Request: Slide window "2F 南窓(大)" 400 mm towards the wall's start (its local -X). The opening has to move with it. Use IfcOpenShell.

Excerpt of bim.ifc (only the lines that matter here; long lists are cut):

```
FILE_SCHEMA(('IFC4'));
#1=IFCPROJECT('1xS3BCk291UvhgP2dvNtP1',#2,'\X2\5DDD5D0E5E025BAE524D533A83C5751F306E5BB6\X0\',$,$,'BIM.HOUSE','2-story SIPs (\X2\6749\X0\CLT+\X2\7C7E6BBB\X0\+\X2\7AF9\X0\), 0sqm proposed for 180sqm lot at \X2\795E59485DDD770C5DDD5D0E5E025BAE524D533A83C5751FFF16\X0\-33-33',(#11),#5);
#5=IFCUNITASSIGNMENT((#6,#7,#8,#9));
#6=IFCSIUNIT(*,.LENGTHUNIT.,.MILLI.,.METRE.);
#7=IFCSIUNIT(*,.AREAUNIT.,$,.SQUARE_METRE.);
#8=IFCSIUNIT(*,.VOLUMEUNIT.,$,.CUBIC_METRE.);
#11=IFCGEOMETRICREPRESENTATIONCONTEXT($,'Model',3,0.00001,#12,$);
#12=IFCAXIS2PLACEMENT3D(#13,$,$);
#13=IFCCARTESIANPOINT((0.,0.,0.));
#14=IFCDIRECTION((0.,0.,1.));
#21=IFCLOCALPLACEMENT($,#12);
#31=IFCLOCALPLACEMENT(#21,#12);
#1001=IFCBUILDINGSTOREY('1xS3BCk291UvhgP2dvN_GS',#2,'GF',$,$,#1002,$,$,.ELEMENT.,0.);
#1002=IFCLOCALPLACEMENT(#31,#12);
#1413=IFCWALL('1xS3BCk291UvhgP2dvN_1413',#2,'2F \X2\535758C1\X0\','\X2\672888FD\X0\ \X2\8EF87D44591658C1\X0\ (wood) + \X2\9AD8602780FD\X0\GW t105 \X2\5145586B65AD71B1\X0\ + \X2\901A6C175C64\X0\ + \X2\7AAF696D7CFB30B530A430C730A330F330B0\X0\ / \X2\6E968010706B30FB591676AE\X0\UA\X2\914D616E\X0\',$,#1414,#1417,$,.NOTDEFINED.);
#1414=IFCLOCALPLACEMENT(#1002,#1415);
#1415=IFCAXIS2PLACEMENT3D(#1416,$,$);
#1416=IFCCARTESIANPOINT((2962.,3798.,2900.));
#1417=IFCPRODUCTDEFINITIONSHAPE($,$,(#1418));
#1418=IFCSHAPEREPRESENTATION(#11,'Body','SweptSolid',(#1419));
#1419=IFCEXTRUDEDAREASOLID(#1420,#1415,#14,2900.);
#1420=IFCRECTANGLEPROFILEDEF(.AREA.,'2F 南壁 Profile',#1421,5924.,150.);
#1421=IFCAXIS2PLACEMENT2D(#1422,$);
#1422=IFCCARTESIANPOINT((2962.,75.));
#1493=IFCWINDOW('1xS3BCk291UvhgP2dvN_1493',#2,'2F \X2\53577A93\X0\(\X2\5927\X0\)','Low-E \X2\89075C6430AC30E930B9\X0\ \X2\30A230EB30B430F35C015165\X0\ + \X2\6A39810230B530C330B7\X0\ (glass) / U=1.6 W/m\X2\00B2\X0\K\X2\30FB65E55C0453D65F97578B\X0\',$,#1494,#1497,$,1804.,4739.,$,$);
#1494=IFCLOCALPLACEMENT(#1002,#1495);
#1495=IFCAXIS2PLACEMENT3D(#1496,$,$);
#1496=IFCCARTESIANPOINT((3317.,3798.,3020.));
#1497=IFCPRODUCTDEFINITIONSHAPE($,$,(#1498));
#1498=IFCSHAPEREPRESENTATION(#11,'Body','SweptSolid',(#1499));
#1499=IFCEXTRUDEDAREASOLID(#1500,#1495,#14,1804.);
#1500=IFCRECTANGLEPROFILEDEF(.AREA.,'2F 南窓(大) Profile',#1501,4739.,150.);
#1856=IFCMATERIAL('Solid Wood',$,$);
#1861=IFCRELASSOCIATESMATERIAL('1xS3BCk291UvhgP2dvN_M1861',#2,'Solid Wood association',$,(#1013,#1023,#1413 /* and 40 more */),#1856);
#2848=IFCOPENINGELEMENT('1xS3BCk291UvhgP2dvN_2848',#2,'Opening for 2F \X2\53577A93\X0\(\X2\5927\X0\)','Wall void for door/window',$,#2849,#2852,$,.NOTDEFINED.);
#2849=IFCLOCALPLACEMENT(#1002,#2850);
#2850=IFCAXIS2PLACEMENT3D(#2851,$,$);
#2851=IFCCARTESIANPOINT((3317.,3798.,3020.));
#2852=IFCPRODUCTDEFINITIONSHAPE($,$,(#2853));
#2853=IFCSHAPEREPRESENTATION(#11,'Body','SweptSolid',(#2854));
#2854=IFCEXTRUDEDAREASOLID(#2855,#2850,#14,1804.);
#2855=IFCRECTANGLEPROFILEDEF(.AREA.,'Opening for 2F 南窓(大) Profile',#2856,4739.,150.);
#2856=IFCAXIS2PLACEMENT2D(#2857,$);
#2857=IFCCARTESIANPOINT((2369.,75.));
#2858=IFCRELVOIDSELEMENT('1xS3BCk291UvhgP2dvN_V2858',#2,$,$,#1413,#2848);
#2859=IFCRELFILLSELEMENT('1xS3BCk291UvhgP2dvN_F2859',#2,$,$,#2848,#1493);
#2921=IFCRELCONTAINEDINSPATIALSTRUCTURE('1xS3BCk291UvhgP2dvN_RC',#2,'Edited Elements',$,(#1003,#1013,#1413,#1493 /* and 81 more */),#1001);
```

```python
import ifcopenshell
import ifcopenshell.api.geometry
import ifcopenshell.util.placement
import ifcopenshell.util.unit

model = ifcopenshell.open("bim.ifc")
unit_scale = ifcopenshell.util.unit.calculate_unit_scale(model)

window = model.by_guid("1xS3BCk291UvhgP2dvN_1493")
opening = window.FillsVoids[0].RelatingOpeningElement
wall = opening.VoidsElements[0].RelatingBuildingElement

wall_matrix = ifcopenshell.util.placement.get_local_placement(wall.ObjectPlacement)
shift = wall_matrix[:3, 0] * -0.4 / unit_scale
before = ifcopenshell.util.placement.get_local_placement(window.ObjectPlacement)[:3, 3].copy()

# The window is not placed relative to its opening, so move both.
for product in (opening, window):
    matrix = ifcopenshell.util.placement.get_local_placement(product.ObjectPlacement)
    matrix[:3, 3] += shift
    ifcopenshell.api.geometry.edit_object_placement(model, product=product, matrix=matrix, is_si=False)

after = ifcopenshell.util.placement.get_local_placement(window.ObjectPlacement)[:3, 3]
print("window moved by", (after - before).round(3) + 0.0)

model.write("bim-out.ifc")
```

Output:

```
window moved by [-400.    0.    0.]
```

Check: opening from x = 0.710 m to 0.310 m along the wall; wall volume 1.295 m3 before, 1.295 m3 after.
